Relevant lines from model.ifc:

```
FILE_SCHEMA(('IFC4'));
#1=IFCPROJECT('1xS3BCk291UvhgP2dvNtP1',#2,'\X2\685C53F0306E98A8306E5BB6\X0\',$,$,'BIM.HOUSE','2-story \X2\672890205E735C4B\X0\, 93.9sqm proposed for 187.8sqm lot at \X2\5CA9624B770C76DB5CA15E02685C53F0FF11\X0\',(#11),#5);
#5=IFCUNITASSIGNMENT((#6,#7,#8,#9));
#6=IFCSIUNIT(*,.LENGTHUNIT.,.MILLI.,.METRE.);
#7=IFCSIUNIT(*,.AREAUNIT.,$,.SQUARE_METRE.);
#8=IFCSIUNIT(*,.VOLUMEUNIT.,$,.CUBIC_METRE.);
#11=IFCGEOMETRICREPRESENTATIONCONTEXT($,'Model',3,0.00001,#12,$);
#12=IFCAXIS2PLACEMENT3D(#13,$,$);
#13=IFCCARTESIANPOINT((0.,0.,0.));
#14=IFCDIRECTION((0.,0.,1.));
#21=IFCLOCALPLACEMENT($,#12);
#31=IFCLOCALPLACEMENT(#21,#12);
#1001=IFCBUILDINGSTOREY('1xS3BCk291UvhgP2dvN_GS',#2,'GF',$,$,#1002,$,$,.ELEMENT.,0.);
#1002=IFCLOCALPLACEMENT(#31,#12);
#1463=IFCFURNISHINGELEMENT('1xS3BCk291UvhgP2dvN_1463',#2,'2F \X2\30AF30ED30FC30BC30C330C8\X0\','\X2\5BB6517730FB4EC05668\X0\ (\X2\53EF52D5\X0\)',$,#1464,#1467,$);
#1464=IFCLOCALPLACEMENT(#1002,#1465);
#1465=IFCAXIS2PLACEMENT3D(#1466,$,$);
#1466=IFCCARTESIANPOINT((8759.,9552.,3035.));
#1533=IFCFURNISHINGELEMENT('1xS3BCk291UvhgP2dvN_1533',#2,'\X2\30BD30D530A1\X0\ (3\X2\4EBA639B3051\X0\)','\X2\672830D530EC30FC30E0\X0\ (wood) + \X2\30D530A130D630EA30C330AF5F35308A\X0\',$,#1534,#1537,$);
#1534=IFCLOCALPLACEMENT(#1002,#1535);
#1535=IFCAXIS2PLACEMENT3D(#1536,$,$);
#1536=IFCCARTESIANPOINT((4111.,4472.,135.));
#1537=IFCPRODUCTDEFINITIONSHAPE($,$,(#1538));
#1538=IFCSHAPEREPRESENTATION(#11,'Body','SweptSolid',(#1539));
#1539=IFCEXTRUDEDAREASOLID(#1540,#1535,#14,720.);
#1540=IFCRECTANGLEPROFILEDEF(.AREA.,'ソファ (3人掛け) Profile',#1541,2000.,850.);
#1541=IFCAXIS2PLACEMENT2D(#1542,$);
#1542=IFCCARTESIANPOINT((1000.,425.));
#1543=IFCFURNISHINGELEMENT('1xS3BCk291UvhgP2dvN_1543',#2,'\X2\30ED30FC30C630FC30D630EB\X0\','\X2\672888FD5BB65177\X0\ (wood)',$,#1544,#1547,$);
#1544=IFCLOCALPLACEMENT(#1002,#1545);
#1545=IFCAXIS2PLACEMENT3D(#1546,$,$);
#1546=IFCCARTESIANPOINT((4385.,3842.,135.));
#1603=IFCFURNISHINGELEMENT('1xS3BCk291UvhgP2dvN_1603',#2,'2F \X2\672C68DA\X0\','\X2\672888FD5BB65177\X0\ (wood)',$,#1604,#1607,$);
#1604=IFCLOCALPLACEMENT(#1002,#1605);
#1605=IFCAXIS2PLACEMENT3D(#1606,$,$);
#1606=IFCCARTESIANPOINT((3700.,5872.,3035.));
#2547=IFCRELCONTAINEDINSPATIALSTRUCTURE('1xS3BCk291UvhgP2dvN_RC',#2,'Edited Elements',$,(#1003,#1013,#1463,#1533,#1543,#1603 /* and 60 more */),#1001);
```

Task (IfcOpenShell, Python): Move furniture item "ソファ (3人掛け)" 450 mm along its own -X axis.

```python
import ifcopenshell
import ifcopenshell.api.geometry
import ifcopenshell.util.placement

model = ifcopenshell.open("model.ifc")

item = model.by_guid("1xS3BCk291UvhgP2dvN_1533")
matrix = ifcopenshell.util.placement.get_local_placement(item.ObjectPlacement)
matrix[:3, 3] -= matrix[:3, 0] * 450.0
ifcopenshell.api.geometry.edit_object_placement(model, product=item, matrix=matrix, is_si=False)

print(ifcopenshell.util.placement.get_local_placement(item.ObjectPlacement).round(3) + 0.0)

model.write("model-out.ifc")
```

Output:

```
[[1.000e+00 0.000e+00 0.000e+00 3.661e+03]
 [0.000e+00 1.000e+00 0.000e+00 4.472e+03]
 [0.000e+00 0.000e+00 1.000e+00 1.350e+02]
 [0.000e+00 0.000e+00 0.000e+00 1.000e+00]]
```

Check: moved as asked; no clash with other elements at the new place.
